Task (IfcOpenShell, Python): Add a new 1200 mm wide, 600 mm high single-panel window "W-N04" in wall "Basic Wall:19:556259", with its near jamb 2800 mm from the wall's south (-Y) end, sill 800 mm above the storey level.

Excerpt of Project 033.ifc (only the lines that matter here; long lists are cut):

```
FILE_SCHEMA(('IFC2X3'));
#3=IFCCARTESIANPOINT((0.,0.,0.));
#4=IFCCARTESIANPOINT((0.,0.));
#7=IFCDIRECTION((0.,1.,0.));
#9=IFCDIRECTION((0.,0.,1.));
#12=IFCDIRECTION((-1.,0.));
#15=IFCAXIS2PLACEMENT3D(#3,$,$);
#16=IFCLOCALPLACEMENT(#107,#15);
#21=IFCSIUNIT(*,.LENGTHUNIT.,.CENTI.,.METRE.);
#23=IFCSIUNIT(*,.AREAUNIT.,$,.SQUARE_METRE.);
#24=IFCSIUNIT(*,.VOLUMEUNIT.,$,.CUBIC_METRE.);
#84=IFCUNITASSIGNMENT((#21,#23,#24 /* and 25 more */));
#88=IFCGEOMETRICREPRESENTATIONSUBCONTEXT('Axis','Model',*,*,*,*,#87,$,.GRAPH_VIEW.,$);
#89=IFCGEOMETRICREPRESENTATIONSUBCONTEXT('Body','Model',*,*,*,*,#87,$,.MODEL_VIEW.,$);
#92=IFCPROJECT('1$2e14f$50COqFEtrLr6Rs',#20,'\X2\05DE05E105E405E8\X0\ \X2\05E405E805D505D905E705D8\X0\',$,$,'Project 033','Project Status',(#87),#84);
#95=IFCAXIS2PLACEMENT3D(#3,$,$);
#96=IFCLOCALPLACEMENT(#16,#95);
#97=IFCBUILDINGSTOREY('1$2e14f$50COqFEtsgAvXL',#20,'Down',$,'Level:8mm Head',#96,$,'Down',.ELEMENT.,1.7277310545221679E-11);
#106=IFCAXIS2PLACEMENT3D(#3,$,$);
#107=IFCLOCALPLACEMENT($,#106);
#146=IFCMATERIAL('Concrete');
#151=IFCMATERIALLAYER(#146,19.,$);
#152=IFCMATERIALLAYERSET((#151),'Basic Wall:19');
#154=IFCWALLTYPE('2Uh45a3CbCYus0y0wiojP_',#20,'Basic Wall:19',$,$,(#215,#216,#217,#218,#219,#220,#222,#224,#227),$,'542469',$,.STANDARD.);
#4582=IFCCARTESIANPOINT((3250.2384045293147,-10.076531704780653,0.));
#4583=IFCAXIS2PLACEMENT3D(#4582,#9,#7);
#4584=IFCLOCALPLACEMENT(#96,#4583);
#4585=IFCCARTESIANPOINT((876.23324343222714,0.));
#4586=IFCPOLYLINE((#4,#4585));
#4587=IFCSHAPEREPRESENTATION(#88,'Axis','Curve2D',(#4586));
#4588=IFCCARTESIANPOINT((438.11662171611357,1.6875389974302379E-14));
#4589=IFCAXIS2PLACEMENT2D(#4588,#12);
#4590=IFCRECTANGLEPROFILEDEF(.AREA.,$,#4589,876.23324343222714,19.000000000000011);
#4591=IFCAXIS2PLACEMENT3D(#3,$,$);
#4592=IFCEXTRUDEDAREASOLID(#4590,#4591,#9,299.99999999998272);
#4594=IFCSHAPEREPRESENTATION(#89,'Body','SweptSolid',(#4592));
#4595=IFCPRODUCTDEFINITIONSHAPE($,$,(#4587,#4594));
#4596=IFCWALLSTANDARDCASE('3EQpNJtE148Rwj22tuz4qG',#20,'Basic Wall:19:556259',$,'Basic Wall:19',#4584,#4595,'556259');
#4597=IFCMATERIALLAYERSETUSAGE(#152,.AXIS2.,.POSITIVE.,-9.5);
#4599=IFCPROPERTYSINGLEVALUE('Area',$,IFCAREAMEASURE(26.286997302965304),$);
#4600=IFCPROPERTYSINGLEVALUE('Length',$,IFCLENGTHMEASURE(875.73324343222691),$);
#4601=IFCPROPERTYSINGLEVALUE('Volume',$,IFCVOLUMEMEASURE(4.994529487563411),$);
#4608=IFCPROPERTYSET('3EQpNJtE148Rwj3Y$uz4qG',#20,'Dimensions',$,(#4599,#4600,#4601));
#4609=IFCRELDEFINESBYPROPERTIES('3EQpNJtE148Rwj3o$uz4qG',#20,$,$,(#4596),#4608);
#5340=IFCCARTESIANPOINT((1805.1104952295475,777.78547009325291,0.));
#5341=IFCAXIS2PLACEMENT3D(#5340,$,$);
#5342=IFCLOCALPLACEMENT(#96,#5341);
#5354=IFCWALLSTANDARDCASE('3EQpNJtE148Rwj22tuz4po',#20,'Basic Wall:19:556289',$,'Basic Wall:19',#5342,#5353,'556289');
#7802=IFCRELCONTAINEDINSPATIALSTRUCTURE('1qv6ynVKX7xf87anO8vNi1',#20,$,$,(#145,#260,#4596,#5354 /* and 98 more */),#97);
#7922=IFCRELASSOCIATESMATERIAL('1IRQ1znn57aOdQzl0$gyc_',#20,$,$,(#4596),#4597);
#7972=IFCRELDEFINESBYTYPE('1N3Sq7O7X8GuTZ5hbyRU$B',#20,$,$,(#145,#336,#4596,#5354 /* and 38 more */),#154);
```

```python
import numpy as np
import ifcopenshell
import ifcopenshell.api.feature
import ifcopenshell.api.geometry
import ifcopenshell.api.pset
import ifcopenshell.api.root
import ifcopenshell.api.spatial
import ifcopenshell.api.type
import ifcopenshell.geom
import ifcopenshell.util.element
import ifcopenshell.util.placement
import ifcopenshell.util.representation
import ifcopenshell.util.shape
import ifcopenshell.util.unit

model = ifcopenshell.open("Project 033.ifc")
unit_scale = ifcopenshell.util.unit.calculate_unit_scale(model)
area_scale = ifcopenshell.util.unit.calculate_unit_scale(model, "AREAUNIT")
volume_scale = ifcopenshell.util.unit.calculate_unit_scale(model, "VOLUMEUNIT")
settings = ifcopenshell.geom.settings()


def volume(element):
    """Net volume in cubic metres, openings subtracted."""
    shape = ifcopenshell.geom.create_shape(settings, element)
    return ifcopenshell.util.shape.get_volume(shape.geometry)


wall = model.by_id(4596)
storey = ifcopenshell.util.element.get_container(wall, ifc_class="IfcBuildingStorey")
context = ifcopenshell.util.representation.get_context(model, "Model", "Body", "MODEL_VIEW")
before = volume(wall)

width, height, from_end, sill = 1.2, 0.6, 2.8, 0.8  # metres

# The wall runs along its own X axis, and the end named is its -X end.
wall_shape = ifcopenshell.geom.create_shape(settings, wall)
x, y, z = ifcopenshell.util.shape.get_vertices(wall_shape.geometry).T
start = x.min() + from_end
face, thickness = float(y.min()), float(y.max() - y.min())
wall_matrix = ifcopenshell.util.placement.get_local_placement(wall.ObjectPlacement)
level = ifcopenshell.util.placement.get_local_placement(storey.ObjectPlacement)[2, 3]


def in_wall(x, y):
    """Placement at x, y metres in the wall's axes, at sill height."""
    matrix = wall_matrix.copy()
    matrix[:, 3] = wall_matrix @ np.array([x / unit_scale, y / unit_scale, 0.0, 1.0])
    matrix[2, 3] = level + sill / unit_scale
    return matrix


# Opening: a box that overshoots both wall faces by 50 mm.
opening = ifcopenshell.api.root.create_entity(model, ifc_class="IfcOpeningElement")
box = ifcopenshell.api.geometry.add_wall_representation(
    model, context=context, length=width, height=height, thickness=thickness + 0.1
)
ifcopenshell.api.geometry.assign_representation(model, product=opening, representation=box)
ifcopenshell.api.geometry.edit_object_placement(model, product=opening, matrix=in_wall(start, face - 0.05), is_si=False)
ifcopenshell.api.feature.add_feature(model, feature=opening, element=wall)

window = ifcopenshell.api.root.create_entity(model, ifc_class="IfcWindow", name="W-N04")
window.OverallWidth, window.OverallHeight = width / unit_scale, height / unit_scale
body = ifcopenshell.api.geometry.add_window_representation(
    model,
    context=context,
    overall_width=window.OverallWidth,
    overall_height=window.OverallHeight,
    partition_type="SINGLE_PANEL",
)
ifcopenshell.api.geometry.assign_representation(model, product=window, representation=body)
ifcopenshell.api.spatial.assign_container(model, products=[window], relating_structure=storey)
fills = ifcopenshell.api.feature.add_filling(model, opening=opening, element=window)
fills.OwnerHistory = window.OwnerHistory  # required in IFC2X3

# IFC2X3 keeps the operation on the window style.
style = ifcopenshell.api.root.create_entity(model, ifc_class="IfcWindowStyle", name="W-N04")
style.OperationType, style.ConstructionType = "SINGLE_PANEL", "NOTDEFINED"
style.ParameterTakesPrecedence = style.Sizeable = False
ifcopenshell.api.type.assign_type(model, related_objects=[window], relating_type=style)

# Centre the window in the wall's thickness.
ifcopenshell.api.geometry.edit_object_placement(model, product=window, matrix=in_wall(start, face), is_si=False)
window_shape = ifcopenshell.geom.create_shape(settings, window)
depth = ifcopenshell.util.shape.get_vertices(window_shape.geometry)[:, 1]
offset = face + thickness / 2 - (depth.min() + depth.max()) / 2
ifcopenshell.api.geometry.edit_object_placement(model, product=window, matrix=in_wall(start, offset), is_si=False)

after = volume(wall)

# Update the wall's stored quantities.
pset = model.by_id(ifcopenshell.util.element.get_pset(wall, "Dimensions", should_inherit=False)["id"])
ifcopenshell.api.pset.edit_pset(model, pset=pset, properties={
    "Area": model.create_entity("IfcAreaMeasure", after / thickness / area_scale),
    "Volume": model.create_entity("IfcVolumeMeasure", after / volume_scale),
})

print(f"wall volume {before:.3f} -> {after:.3f} m3")

model.write("Project 033-out.ifc")
```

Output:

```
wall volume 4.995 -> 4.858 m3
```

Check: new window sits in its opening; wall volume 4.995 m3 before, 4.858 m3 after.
